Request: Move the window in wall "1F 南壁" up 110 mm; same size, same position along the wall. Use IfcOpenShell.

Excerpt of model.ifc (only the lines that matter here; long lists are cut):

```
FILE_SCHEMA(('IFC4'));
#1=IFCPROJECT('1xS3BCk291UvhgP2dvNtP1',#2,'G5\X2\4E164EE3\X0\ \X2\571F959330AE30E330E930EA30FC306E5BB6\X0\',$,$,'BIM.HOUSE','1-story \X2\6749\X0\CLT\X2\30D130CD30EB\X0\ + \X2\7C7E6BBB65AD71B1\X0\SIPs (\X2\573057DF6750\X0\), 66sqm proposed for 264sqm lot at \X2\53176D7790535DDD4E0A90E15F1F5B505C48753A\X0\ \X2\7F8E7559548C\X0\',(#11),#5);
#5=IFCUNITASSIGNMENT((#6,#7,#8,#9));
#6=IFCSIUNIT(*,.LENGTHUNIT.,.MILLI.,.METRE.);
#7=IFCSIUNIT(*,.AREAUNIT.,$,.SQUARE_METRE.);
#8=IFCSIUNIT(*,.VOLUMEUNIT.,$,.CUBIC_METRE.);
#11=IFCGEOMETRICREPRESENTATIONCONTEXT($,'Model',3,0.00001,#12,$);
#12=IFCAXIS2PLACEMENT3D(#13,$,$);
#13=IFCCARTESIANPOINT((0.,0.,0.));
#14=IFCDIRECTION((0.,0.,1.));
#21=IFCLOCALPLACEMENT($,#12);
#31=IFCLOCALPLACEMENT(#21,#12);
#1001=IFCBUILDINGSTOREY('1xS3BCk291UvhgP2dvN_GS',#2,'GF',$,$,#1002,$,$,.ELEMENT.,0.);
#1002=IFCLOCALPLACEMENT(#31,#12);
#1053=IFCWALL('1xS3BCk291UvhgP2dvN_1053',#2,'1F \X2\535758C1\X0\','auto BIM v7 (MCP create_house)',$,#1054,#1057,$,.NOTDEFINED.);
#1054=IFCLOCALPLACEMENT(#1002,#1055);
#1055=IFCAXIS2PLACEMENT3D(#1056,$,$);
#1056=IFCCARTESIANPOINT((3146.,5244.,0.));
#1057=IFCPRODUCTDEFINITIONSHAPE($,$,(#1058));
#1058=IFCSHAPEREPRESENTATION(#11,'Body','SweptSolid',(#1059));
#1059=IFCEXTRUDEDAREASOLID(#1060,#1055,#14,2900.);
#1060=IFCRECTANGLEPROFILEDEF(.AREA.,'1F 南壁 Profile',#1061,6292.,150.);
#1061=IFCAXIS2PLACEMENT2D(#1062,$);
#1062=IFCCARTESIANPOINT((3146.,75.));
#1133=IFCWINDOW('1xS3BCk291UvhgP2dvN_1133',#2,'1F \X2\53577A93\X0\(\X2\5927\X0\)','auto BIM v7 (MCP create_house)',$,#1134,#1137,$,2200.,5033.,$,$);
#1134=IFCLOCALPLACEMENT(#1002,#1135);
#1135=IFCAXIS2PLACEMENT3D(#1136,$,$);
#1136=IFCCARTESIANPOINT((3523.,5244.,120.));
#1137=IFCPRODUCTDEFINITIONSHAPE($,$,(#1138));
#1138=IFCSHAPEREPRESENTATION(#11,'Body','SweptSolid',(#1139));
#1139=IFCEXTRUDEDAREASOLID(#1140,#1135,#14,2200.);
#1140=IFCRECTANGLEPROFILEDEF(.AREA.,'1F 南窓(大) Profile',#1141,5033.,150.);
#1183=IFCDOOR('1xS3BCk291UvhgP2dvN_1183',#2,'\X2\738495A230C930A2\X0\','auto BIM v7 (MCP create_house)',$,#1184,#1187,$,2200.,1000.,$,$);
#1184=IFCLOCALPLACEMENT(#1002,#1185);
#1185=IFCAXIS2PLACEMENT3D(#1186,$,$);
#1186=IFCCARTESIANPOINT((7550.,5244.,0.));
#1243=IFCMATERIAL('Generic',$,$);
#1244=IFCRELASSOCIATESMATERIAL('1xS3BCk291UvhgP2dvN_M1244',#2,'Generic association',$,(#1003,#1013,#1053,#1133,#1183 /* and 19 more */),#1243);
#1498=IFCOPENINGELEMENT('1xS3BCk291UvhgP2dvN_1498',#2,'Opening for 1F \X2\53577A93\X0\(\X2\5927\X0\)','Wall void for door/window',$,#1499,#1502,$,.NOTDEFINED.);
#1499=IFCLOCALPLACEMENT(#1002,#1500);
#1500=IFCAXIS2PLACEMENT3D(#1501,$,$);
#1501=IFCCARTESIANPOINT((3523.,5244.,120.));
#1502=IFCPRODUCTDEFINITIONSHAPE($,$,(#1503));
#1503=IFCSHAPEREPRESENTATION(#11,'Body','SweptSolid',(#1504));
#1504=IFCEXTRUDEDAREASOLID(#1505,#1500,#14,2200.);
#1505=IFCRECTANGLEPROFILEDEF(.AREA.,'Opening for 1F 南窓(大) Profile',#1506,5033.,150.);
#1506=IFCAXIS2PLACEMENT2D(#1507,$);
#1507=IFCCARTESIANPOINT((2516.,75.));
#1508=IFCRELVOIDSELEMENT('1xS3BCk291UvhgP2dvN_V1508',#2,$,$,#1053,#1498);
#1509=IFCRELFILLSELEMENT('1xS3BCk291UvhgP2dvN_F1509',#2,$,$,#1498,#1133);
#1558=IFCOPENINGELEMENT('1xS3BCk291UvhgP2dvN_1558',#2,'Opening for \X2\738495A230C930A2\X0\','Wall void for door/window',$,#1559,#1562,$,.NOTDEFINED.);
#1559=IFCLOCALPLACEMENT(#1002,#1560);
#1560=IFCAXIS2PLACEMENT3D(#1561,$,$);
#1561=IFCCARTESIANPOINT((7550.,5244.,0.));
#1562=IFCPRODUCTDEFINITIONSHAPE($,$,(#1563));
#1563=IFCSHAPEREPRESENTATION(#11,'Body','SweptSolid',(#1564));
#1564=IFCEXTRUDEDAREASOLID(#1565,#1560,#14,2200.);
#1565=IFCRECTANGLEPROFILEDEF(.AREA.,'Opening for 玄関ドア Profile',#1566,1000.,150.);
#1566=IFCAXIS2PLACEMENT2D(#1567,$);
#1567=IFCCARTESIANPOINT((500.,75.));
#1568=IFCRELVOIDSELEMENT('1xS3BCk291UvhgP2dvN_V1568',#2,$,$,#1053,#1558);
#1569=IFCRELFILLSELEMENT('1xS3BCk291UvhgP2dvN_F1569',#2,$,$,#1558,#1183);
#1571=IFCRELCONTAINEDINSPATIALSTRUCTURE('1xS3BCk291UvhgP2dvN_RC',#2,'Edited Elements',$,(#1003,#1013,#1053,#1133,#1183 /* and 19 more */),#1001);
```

```python
import numpy as np
import ifcopenshell
import ifcopenshell.api.geometry
import ifcopenshell.util.placement
import ifcopenshell.util.unit

model = ifcopenshell.open("model.ifc")
unit_scale = ifcopenshell.util.unit.calculate_unit_scale(model)

window = model.by_guid("1xS3BCk291UvhgP2dvN_1133")
opening = window.FillsVoids[0].RelatingOpeningElement
dz = 0.11 / unit_scale

shift = np.array([0.0, 0.0, dz])
# The window is not placed relative to its opening, so move both.
for product in (opening, window):
    matrix = ifcopenshell.util.placement.get_local_placement(product.ObjectPlacement)
    matrix[:3, 3] += shift
    ifcopenshell.api.geometry.edit_object_placement(model, product=product, matrix=matrix, is_si=False)

print(f"moved by {dz * unit_scale:+.3f} m")

model.write("model_updated.ifc")
```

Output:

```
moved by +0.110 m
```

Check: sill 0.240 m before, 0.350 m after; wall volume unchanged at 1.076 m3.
